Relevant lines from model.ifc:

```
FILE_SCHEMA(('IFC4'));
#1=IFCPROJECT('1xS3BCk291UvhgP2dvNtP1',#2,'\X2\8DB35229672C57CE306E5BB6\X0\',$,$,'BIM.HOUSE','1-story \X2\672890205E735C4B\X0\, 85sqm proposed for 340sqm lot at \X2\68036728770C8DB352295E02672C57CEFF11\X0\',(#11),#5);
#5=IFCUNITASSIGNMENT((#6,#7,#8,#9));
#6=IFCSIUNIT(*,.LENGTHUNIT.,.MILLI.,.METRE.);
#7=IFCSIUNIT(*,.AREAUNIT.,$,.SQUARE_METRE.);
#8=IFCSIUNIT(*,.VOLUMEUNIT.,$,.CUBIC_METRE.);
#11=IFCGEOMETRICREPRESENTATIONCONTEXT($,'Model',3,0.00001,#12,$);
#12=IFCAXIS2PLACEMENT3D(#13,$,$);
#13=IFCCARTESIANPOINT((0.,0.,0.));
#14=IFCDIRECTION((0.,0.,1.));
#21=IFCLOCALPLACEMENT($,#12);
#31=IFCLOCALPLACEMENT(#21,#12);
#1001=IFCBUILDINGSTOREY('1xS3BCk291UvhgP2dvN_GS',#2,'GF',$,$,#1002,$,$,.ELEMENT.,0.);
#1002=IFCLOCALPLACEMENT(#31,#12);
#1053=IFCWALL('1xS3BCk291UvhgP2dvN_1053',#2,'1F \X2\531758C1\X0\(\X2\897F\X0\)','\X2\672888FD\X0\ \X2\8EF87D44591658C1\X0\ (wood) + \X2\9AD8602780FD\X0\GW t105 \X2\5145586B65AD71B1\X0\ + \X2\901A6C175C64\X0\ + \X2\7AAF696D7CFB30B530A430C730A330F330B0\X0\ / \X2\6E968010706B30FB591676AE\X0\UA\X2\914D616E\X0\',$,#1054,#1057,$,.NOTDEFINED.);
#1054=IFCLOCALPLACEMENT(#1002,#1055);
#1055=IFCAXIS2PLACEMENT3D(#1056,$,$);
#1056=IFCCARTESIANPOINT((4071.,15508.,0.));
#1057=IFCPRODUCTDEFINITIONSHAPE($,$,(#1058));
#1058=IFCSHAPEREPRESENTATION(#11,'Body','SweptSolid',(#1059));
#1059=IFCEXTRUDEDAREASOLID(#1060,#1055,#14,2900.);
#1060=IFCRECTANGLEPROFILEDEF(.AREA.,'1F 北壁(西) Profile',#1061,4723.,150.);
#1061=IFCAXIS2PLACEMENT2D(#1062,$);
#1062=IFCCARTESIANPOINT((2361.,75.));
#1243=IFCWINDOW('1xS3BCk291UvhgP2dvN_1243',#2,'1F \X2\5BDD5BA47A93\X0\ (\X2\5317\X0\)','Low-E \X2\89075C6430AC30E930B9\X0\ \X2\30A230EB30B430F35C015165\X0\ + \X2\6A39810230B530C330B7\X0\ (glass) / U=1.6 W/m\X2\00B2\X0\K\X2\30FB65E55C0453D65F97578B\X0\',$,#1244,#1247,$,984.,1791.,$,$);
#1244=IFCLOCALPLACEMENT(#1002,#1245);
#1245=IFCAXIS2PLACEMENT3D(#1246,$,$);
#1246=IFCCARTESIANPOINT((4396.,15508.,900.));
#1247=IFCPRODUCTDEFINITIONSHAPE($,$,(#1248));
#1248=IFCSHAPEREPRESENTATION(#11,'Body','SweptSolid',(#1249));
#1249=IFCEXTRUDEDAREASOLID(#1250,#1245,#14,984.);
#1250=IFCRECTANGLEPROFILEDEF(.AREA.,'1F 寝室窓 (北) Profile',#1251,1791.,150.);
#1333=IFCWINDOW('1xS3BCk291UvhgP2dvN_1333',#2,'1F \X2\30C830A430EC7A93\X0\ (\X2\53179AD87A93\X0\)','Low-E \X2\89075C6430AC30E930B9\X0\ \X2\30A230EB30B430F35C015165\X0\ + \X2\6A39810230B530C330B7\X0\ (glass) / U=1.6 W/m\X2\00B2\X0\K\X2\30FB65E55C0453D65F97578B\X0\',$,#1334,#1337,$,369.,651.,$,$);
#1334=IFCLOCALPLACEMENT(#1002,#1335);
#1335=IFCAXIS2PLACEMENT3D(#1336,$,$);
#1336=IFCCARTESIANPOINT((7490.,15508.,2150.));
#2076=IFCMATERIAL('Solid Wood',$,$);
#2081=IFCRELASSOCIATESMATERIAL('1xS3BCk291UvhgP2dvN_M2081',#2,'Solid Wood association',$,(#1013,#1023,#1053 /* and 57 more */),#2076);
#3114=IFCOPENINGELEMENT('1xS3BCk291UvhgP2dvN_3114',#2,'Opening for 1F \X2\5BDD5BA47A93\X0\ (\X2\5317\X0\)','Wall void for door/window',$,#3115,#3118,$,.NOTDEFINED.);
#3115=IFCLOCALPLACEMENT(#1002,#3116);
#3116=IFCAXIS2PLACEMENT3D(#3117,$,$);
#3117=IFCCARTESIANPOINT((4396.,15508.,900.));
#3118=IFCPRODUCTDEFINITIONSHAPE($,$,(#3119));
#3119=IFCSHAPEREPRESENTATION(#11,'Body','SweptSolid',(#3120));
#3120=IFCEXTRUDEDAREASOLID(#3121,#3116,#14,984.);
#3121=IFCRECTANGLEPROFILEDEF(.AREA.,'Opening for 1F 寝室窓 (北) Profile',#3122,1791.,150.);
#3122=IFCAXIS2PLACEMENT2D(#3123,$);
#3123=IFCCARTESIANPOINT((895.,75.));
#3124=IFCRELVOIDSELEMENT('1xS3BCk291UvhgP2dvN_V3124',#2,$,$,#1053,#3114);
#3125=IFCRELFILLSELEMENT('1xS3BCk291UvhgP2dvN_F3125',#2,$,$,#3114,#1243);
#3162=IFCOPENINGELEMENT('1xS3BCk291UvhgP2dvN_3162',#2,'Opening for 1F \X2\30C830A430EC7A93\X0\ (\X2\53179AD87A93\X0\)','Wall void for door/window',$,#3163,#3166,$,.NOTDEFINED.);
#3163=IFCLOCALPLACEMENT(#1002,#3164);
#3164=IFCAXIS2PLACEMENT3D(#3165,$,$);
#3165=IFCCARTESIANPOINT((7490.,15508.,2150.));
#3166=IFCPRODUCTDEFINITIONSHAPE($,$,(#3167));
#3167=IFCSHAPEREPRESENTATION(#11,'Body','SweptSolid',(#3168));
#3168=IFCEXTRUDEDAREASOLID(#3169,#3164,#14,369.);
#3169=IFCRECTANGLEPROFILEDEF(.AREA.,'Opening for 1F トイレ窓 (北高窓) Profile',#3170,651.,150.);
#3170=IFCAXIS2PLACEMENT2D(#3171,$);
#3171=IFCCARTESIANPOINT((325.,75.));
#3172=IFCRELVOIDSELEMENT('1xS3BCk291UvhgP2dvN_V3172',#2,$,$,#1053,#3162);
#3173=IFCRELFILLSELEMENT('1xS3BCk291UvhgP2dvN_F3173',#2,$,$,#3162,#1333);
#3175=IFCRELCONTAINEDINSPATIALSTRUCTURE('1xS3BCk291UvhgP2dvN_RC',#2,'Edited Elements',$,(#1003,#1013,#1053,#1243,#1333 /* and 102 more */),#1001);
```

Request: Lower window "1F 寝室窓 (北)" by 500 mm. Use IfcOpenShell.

```python
import numpy as np
import ifcopenshell
import ifcopenshell.api.geometry
import ifcopenshell.util.placement
import ifcopenshell.util.unit

model = ifcopenshell.open("model.ifc")
unit_scale = ifcopenshell.util.unit.calculate_unit_scale(model)

window = model.by_id(1243)
opening = window.FillsVoids[0].RelatingOpeningElement
dz = -0.5 / unit_scale

shift = np.array([0.0, 0.0, dz])
# The window is not placed relative to its opening, so move both.
for product in (opening, window):
    matrix = ifcopenshell.util.placement.get_local_placement(product.ObjectPlacement)
    matrix[:3, 3] += shift
    ifcopenshell.api.geometry.edit_object_placement(model, product=product, matrix=matrix, is_si=False)

print(f"moved by {dz * unit_scale:+.3f} m")

model.write("model_updated.ifc")
```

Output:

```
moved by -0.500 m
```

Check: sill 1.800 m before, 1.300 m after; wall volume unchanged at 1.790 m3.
